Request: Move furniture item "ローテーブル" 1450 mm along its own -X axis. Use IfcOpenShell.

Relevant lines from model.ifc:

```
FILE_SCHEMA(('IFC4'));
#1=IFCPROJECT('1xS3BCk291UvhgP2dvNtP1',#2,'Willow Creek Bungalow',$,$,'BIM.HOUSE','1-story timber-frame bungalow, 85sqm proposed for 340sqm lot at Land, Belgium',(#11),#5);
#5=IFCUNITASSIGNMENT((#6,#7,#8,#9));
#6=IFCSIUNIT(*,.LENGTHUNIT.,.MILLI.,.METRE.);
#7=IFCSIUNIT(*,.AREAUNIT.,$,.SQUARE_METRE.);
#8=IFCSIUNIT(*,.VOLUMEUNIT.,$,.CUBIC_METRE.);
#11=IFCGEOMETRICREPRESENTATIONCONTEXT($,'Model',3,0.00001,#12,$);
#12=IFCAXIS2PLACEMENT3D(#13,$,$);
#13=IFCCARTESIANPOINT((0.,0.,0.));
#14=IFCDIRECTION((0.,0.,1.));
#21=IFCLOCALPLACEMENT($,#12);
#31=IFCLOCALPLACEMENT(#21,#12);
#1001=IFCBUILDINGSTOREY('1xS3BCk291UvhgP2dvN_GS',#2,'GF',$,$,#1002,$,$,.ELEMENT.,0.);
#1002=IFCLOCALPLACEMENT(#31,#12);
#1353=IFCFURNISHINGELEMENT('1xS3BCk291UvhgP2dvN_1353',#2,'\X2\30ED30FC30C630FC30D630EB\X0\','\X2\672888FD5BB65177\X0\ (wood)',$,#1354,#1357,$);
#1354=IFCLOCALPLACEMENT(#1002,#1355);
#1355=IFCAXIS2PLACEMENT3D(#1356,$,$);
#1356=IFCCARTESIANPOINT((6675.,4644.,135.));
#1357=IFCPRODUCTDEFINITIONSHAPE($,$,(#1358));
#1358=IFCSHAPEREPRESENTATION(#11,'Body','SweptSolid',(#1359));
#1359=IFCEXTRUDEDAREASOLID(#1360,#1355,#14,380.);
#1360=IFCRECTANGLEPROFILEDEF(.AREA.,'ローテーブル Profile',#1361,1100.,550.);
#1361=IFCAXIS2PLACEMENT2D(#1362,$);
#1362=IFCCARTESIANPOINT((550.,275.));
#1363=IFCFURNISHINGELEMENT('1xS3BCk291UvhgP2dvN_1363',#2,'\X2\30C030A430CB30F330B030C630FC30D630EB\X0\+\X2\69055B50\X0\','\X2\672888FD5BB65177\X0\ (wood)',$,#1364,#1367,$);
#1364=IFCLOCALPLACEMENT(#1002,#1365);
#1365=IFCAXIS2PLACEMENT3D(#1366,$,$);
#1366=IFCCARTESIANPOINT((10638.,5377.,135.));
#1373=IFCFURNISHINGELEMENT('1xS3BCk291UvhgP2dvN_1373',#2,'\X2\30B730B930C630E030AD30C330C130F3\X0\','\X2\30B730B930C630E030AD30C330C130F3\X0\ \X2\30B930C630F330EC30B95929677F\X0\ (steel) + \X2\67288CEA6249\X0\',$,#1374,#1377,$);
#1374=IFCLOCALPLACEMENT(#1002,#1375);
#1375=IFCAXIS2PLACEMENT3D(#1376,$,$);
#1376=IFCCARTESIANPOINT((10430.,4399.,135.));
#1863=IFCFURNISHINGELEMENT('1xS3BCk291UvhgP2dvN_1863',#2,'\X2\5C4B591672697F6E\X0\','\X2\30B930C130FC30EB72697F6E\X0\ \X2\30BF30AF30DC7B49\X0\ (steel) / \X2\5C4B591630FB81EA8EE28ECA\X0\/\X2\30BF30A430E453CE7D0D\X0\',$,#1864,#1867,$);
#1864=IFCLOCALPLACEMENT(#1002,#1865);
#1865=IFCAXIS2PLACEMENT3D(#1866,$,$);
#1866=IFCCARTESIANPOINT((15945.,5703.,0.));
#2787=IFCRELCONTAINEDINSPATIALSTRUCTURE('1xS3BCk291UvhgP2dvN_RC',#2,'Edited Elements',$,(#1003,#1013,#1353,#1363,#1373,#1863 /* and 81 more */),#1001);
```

```python
import ifcopenshell
import ifcopenshell.api.geometry
import ifcopenshell.util.placement

model = ifcopenshell.open("model.ifc")

item = model.by_id(1353)
matrix = ifcopenshell.util.placement.get_local_placement(item.ObjectPlacement)
matrix[:3, 3] -= matrix[:3, 0] * 1450.0
ifcopenshell.api.geometry.edit_object_placement(model, product=item, matrix=matrix, is_si=False)

print(ifcopenshell.util.placement.get_local_placement(item.ObjectPlacement).round(3) + 0.0)

model.write("model_edited.ifc")
```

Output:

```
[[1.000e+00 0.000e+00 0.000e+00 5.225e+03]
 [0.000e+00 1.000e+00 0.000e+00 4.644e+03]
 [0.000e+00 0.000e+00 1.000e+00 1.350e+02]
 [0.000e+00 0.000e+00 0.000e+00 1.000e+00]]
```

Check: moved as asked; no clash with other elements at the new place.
